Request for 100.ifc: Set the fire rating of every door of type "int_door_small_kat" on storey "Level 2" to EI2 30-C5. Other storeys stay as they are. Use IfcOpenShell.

First a look at what the model holds.

```python
import ifcopenshell
import ifcopenshell.util.element

model = ifcopenshell.open("100.ifc")
print(model.schema)
storey = next(s for s in model.by_type("IfcBuildingStorey") if s.Name == "Level 2")
doors = [e for e in ifcopenshell.util.element.get_decomposition(storey) if e.is_a("IfcDoor")]
seen = {}
for e in doors:
    element_type = ifcopenshell.util.element.get_type(e)
    key = (element_type.Name if element_type != e and element_type else None, ifcopenshell.util.element.get_pset(e, "Pset_DoorCommon", "FireRating"))
    seen[key] = seen.get(key, 0) + 1
for (name, value), count in sorted(seen.items(), key=str):
    print(count, "x", name, "|", value)
```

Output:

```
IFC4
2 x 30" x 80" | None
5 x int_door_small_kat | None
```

```python
import ifcopenshell
import ifcopenshell.api.pset
import ifcopenshell.util.element

model = ifcopenshell.open("100.ifc")

storey = next(s for s in model.by_type("IfcBuildingStorey") if s.Name == "Level 2")
doors = [e for e in ifcopenshell.util.element.get_decomposition(storey) if e.is_a("IfcDoor")]

count = 0
for e in doors:
    element_type = ifcopenshell.util.element.get_type(e)
    if element_type in (None, e) or element_type.Name != "int_door_small_kat":
        continue
    # add_pset returns the element's existing set when there is one.
    pset = ifcopenshell.api.pset.add_pset(model, product=e, name="Pset_DoorCommon")
    ifcopenshell.api.pset.edit_pset(model, pset=pset, properties={"FireRating": "EI2 30-C5"})
    count += 1

print(count, "doors updated")

model.write("100-out.ifc")
```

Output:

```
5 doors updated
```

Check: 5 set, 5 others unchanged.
